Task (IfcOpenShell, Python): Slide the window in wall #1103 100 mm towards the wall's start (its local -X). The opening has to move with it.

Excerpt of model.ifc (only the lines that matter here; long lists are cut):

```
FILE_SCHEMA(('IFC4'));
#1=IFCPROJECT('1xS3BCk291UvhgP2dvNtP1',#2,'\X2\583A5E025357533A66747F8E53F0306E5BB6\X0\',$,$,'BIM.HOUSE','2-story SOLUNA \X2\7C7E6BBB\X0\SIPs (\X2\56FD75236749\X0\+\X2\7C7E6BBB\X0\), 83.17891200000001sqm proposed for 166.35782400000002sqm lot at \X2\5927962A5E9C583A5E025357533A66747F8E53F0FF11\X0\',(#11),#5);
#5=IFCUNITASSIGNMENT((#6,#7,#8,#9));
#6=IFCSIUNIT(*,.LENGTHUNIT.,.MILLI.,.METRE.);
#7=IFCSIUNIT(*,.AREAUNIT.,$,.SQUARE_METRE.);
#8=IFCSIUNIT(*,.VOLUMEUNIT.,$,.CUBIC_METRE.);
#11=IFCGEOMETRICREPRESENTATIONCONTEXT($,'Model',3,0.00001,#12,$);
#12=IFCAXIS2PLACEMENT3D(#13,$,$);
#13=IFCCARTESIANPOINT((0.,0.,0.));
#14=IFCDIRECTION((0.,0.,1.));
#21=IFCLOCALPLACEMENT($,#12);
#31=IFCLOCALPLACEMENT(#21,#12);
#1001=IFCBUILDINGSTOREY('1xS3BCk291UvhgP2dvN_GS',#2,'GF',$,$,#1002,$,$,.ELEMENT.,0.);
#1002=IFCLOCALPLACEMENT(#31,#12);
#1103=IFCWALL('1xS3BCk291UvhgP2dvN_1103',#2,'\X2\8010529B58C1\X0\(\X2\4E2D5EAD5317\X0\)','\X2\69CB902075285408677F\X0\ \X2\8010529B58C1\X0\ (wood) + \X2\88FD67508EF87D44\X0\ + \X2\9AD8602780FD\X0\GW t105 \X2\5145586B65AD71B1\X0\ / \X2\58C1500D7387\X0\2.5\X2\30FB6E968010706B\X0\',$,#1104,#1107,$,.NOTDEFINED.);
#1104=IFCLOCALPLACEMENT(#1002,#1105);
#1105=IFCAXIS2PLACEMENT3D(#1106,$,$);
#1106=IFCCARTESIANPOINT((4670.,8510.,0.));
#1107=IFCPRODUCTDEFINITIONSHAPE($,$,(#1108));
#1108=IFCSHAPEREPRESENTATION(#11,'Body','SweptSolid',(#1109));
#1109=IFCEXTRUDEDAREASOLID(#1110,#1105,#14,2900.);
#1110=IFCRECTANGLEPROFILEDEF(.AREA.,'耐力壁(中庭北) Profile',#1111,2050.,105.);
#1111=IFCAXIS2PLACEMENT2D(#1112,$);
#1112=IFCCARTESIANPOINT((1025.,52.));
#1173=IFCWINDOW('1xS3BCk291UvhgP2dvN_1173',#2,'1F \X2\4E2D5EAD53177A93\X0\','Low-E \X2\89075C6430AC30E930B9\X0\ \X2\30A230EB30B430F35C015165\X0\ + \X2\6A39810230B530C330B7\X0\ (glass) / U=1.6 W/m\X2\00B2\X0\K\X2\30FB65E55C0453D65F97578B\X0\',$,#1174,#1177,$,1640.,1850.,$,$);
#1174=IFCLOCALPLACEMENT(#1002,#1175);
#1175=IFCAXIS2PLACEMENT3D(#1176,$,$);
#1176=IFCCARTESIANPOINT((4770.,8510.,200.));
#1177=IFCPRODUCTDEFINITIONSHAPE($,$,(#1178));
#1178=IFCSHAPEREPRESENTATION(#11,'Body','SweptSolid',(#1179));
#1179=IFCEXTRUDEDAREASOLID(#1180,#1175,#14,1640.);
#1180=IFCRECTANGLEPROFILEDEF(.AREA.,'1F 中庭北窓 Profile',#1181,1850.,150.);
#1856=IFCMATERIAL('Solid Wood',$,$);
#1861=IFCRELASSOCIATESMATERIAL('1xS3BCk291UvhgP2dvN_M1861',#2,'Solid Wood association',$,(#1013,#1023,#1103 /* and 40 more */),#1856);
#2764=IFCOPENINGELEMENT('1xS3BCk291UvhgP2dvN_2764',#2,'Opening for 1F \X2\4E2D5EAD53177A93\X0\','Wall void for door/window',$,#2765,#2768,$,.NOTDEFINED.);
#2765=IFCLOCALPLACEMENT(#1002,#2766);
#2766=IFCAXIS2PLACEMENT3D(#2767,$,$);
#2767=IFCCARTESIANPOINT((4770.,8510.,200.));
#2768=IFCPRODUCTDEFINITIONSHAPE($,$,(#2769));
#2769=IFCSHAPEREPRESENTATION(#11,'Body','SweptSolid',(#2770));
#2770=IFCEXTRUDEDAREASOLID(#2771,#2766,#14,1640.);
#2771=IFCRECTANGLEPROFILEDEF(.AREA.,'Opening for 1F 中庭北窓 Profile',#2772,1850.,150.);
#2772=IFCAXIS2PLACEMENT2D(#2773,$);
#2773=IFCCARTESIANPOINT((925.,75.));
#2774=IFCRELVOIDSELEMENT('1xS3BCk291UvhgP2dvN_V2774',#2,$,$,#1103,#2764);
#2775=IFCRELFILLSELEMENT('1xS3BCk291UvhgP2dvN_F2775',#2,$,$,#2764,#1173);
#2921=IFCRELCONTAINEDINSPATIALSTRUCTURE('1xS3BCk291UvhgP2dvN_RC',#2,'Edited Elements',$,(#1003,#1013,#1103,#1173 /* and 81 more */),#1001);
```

```python
import ifcopenshell
import ifcopenshell.api.geometry
import ifcopenshell.util.placement
import ifcopenshell.util.unit

model = ifcopenshell.open("model.ifc")
unit_scale = ifcopenshell.util.unit.calculate_unit_scale(model)

window = model.by_guid("1xS3BCk291UvhgP2dvN_1173")
opening = window.FillsVoids[0].RelatingOpeningElement
wall = opening.VoidsElements[0].RelatingBuildingElement

wall_matrix = ifcopenshell.util.placement.get_local_placement(wall.ObjectPlacement)
shift = wall_matrix[:3, 0] * -0.1 / unit_scale
before = ifcopenshell.util.placement.get_local_placement(window.ObjectPlacement)[:3, 3].copy()

# The window is not placed relative to its opening, so move both.
for product in (opening, window):
    matrix = ifcopenshell.util.placement.get_local_placement(product.ObjectPlacement)
    matrix[:3, 3] += shift
    ifcopenshell.api.geometry.edit_object_placement(model, product=product, matrix=matrix, is_si=False)

after = ifcopenshell.util.placement.get_local_placement(window.ObjectPlacement)[:3, 3]
print("window moved by", (after - before).round(3) + 0.0)

model.write("model_edited.ifc")
```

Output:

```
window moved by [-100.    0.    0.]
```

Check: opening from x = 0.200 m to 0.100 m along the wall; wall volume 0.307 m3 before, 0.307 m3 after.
